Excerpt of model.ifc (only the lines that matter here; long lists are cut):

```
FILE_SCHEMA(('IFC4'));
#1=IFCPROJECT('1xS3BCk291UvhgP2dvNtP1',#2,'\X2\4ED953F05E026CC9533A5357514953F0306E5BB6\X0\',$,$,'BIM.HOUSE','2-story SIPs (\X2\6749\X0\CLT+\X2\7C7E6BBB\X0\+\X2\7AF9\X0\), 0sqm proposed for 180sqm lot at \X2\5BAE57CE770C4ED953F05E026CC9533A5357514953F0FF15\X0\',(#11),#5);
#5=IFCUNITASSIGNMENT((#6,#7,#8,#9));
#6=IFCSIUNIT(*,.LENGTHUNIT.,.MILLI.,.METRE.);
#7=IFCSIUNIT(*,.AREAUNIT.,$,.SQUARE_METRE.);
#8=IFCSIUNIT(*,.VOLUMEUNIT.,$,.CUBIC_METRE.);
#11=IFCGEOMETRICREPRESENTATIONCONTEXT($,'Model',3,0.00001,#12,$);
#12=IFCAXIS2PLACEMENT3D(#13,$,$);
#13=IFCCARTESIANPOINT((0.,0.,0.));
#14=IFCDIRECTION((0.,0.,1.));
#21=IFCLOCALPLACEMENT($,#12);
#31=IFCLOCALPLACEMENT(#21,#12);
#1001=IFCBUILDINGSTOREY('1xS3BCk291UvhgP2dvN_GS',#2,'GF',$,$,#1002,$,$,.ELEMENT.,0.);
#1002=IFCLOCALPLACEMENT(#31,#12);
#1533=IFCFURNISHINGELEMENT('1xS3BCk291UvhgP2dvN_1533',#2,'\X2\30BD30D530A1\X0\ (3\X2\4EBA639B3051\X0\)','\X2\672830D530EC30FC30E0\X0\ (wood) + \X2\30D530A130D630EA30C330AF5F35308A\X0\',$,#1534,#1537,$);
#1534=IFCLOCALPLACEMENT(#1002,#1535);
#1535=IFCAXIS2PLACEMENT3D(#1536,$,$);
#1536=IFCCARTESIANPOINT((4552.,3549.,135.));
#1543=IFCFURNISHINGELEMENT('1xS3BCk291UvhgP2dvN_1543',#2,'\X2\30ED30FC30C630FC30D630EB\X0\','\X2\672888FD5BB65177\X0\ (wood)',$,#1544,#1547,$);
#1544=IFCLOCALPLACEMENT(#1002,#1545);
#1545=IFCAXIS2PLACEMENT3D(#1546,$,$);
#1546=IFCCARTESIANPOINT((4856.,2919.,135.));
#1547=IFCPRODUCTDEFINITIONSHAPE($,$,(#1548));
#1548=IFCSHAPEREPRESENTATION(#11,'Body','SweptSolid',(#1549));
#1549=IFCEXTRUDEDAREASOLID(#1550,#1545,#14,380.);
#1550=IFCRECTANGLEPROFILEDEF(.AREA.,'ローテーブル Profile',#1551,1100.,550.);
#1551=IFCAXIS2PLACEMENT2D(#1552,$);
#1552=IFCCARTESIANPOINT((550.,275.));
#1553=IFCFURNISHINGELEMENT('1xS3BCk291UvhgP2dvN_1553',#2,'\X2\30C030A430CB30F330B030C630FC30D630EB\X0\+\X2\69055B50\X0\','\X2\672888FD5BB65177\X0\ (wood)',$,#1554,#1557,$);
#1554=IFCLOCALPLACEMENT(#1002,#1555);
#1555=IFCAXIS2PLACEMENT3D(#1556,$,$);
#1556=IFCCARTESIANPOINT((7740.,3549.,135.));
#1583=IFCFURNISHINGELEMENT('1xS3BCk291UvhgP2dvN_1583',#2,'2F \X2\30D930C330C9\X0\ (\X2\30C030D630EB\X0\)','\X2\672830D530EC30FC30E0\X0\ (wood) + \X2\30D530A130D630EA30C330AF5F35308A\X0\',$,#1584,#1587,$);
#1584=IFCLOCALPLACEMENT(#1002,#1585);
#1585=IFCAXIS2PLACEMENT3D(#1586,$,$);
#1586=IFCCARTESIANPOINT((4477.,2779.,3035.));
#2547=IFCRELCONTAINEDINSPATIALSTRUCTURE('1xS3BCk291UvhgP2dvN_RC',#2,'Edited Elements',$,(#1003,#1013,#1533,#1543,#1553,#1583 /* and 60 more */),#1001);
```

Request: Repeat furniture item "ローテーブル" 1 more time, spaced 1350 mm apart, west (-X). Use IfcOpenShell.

```python
import numpy as np
import ifcopenshell
import ifcopenshell.api.geometry
import ifcopenshell.api.root
import ifcopenshell.util.element
import ifcopenshell.util.placement
import ifcopenshell.util.unit

model = ifcopenshell.open("model.ifc")
unit_scale = ifcopenshell.util.unit.calculate_unit_scale(model)


def reuse_history(source, copy):
    """copy_class also copies each property set's owner history, people and application; keep the originals."""
    for rel in copy.IsDefinedBy:
        if rel.is_a("IfcRelDefinesByProperties") and (history := rel.RelatingPropertyDefinition.OwnerHistory):
            rel.RelatingPropertyDefinition.OwnerHistory = source.OwnerHistory
            ifcopenshell.util.element.remove_deep2(model, history)


source = model.by_guid("1xS3BCk291UvhgP2dvN_1543")
base = ifcopenshell.util.placement.get_local_placement(source.ObjectPlacement)
step = np.array([-1.0, 0.0, 0.0]) * 1.35 / unit_scale

for i in range(1, 2):
    copy = ifcopenshell.api.root.copy_class(model, product=source)
    copy.Representation = ifcopenshell.util.element.copy_deep(
        model, source.Representation, exclude=["IfcGeometricRepresentationContext", "IfcRepresentationMap"]
    )
    reuse_history(source, copy)
    matrix = base.copy()
    matrix[:3, 3] += i * step
    print("added at", matrix[:3, 3].round(3) + 0.0)
    ifcopenshell.api.geometry.edit_object_placement(model, product=copy, matrix=matrix, is_si=False)

model.write("model_rev.ifc")
```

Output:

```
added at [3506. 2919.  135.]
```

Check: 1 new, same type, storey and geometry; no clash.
